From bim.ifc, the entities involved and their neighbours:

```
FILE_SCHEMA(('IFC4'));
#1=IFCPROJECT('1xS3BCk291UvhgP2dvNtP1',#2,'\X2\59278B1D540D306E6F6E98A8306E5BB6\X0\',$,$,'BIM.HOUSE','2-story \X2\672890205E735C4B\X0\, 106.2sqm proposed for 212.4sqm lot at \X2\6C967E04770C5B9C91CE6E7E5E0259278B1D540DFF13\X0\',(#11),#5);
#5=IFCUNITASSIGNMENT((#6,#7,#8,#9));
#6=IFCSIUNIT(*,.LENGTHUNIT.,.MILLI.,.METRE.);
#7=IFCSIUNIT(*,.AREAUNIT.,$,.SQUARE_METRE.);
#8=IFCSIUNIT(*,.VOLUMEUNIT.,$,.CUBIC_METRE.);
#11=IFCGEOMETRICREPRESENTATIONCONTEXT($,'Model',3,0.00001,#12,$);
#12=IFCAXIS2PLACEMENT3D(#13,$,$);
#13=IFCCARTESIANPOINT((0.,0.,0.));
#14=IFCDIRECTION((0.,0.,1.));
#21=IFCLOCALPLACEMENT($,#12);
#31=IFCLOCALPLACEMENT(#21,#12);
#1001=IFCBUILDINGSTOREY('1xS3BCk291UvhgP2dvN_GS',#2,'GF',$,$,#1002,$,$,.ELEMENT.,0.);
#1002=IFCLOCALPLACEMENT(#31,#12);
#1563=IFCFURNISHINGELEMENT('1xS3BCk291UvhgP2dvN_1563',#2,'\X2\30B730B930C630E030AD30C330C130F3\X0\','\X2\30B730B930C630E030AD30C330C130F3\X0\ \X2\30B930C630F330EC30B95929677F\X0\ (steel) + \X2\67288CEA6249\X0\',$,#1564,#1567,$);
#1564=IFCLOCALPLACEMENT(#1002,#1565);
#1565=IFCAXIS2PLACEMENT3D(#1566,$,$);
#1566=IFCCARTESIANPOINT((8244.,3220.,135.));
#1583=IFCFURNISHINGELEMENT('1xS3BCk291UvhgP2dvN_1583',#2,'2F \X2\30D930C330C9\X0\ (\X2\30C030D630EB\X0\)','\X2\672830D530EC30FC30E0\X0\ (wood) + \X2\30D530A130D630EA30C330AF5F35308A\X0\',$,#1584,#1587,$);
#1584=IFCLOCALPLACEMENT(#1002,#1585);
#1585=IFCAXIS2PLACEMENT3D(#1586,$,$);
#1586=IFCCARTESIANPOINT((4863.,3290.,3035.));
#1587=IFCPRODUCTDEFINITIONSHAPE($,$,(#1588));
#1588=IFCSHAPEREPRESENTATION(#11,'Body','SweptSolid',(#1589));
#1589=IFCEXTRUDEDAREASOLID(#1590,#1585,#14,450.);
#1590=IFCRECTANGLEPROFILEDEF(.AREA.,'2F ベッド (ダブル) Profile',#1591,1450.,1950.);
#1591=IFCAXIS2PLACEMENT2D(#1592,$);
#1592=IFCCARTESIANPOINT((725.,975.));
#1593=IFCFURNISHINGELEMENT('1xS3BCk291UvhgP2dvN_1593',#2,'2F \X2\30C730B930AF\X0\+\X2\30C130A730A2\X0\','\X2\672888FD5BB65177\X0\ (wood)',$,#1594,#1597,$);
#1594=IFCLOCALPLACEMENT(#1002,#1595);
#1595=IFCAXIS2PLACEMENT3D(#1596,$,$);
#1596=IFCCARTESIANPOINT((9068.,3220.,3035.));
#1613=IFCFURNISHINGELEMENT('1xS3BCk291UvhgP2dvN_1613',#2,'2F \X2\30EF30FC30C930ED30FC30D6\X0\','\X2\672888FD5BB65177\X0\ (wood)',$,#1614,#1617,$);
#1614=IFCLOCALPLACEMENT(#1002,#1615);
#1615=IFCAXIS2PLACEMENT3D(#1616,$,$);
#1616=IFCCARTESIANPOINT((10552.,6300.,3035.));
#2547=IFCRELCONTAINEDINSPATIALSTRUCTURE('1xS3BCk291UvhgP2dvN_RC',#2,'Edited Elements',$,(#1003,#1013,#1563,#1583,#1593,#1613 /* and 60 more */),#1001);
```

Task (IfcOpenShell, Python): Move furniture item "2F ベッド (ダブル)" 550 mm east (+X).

```python
import ifcopenshell
import ifcopenshell.api.geometry
import ifcopenshell.util.placement
import ifcopenshell.util.unit

model = ifcopenshell.open("bim.ifc")
unit_scale = ifcopenshell.util.unit.calculate_unit_scale(model)

item = model.by_id(1583)
matrix = ifcopenshell.util.placement.get_local_placement(item.ObjectPlacement)
matrix[0, 3] += 0.55 / unit_scale
ifcopenshell.api.geometry.edit_object_placement(model, product=item, matrix=matrix, is_si=False)

print(ifcopenshell.util.placement.get_local_placement(item.ObjectPlacement).round(3) + 0.0)

model.write("bim_v2.ifc")
```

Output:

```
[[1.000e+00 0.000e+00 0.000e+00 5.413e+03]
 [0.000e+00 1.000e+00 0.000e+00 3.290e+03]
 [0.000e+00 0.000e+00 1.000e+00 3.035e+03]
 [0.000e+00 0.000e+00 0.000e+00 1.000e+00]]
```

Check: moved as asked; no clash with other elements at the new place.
